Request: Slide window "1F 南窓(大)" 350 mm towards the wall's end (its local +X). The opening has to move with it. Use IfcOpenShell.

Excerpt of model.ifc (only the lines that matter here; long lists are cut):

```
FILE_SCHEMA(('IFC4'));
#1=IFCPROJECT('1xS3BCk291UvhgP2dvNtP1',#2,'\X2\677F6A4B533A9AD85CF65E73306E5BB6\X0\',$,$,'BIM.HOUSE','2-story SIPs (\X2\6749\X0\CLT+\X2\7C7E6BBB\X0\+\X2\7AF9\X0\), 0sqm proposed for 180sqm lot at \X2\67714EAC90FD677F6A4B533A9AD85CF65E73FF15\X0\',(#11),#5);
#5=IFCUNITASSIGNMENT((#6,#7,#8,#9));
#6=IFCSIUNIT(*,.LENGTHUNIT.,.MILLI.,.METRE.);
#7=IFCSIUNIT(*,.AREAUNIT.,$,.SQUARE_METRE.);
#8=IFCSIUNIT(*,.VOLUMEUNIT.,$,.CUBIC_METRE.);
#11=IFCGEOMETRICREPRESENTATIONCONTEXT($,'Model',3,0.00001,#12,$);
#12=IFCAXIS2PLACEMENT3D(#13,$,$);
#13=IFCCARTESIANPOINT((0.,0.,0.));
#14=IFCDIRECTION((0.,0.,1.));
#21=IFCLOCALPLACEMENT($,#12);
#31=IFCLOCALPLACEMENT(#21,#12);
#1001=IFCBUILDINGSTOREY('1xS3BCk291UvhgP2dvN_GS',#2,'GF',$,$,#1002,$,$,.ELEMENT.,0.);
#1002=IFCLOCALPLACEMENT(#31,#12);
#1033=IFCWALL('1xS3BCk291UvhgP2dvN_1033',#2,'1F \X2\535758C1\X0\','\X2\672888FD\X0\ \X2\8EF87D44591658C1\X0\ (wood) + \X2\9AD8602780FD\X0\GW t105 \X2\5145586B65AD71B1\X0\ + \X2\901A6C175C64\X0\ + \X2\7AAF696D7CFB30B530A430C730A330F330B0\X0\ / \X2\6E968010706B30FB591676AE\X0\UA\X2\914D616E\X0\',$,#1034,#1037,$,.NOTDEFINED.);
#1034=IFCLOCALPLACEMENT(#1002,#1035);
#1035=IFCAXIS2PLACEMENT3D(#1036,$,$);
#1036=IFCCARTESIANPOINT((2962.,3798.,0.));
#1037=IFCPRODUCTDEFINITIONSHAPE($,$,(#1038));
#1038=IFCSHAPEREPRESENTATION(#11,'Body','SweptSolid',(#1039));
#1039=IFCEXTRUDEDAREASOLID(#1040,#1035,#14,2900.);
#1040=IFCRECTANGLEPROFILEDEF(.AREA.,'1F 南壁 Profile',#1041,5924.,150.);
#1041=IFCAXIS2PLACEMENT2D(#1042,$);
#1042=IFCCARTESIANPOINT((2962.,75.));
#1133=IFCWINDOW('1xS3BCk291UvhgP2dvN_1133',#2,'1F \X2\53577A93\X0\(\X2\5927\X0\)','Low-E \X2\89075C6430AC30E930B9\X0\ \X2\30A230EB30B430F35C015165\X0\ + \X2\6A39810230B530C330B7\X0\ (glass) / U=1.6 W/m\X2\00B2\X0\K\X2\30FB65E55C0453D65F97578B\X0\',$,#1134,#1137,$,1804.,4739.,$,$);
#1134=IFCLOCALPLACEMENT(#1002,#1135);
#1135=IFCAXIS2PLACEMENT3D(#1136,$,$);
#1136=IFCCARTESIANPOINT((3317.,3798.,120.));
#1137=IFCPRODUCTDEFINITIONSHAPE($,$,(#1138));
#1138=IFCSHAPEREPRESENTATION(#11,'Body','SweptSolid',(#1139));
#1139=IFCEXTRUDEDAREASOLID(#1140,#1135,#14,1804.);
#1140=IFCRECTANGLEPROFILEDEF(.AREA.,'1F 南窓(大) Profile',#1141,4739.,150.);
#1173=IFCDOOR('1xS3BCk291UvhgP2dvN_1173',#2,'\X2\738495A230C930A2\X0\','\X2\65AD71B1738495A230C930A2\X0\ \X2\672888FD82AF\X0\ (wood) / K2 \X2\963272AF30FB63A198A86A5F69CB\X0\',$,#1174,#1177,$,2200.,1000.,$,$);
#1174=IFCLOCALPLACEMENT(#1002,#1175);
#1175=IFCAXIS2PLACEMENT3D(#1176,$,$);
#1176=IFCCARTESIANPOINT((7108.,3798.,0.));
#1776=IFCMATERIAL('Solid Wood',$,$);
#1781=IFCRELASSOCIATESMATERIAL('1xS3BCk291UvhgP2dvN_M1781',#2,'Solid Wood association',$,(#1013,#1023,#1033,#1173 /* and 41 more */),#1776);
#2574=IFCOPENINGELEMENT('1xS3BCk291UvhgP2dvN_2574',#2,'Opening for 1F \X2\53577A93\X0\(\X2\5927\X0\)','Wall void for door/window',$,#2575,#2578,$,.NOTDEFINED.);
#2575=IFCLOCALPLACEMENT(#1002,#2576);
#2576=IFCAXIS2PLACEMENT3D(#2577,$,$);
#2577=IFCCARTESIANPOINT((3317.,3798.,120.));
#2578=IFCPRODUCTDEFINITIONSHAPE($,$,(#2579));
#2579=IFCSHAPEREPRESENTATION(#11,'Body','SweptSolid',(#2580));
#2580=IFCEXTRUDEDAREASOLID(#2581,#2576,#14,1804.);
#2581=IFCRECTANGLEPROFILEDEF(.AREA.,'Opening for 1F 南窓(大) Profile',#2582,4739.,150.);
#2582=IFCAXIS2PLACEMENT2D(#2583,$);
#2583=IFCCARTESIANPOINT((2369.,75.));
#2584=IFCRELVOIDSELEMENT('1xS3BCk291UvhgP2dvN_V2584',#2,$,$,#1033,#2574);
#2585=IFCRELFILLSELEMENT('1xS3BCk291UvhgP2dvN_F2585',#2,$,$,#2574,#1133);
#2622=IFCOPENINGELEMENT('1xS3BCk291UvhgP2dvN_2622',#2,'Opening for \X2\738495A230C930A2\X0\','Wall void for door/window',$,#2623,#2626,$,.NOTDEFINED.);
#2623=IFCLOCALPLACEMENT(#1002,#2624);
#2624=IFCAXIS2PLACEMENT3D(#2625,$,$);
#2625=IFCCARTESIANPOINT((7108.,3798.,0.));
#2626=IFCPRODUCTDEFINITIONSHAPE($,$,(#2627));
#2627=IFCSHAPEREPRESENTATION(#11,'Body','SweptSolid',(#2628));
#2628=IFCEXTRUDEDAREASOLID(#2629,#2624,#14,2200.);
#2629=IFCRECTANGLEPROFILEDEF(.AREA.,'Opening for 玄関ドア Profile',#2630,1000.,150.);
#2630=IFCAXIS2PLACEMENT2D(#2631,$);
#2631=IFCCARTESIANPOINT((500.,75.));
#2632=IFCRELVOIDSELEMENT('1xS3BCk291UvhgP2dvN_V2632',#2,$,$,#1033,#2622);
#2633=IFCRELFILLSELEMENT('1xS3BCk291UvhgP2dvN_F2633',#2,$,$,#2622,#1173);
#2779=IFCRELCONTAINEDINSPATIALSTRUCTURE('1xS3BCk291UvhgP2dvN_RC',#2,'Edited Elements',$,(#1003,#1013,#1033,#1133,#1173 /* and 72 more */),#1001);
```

```python
import ifcopenshell
import ifcopenshell.api.geometry
import ifcopenshell.util.placement
import ifcopenshell.util.unit

model = ifcopenshell.open("model.ifc")
unit_scale = ifcopenshell.util.unit.calculate_unit_scale(model)

window = model.by_guid("1xS3BCk291UvhgP2dvN_1133")
opening = window.FillsVoids[0].RelatingOpeningElement
wall = opening.VoidsElements[0].RelatingBuildingElement

wall_matrix = ifcopenshell.util.placement.get_local_placement(wall.ObjectPlacement)
shift = wall_matrix[:3, 0] * 0.35 / unit_scale
before = ifcopenshell.util.placement.get_local_placement(window.ObjectPlacement)[:3, 3].copy()

# The window is not placed relative to its opening, so move both.
for product in (opening, window):
    matrix = ifcopenshell.util.placement.get_local_placement(product.ObjectPlacement)
    matrix[:3, 3] += shift
    ifcopenshell.api.geometry.edit_object_placement(model, product=product, matrix=matrix, is_si=False)

after = ifcopenshell.util.placement.get_local_placement(window.ObjectPlacement)[:3, 3]
print("window moved by", (after - before).round(3) + 0.0)

model.write("model_updated.ifc")
```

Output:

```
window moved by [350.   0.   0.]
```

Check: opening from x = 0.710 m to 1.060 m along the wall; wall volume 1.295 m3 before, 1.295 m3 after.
